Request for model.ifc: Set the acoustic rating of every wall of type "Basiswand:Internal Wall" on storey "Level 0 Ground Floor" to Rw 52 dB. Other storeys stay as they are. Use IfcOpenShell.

First a look at what the model holds.

```python
import ifcopenshell
import ifcopenshell.util.element

model = ifcopenshell.open("model.ifc")
print(model.schema)
storey = next(s for s in model.by_type("IfcBuildingStorey") if s.Name == "Level 0 Ground Floor")
walls = [e for e in ifcopenshell.util.element.get_decomposition(storey) if e.is_a("IfcWall")]
seen = {}
for e in walls:
    element_type = ifcopenshell.util.element.get_type(e)
    key = (element_type.Name if element_type != e and element_type else None, ifcopenshell.util.element.get_pset(e, "Pset_WallCommon", "AcousticRating"))
    seen[key] = seen.get(key, 0) + 1
for (name, value), count in sorted(seen.items(), key=str):
    print(count, "x", name, "|", value)
```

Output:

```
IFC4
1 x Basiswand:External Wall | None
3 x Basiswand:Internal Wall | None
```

```python
import ifcopenshell
import ifcopenshell.api.pset
import ifcopenshell.util.element

model = ifcopenshell.open("model.ifc")

storey = next(s for s in model.by_type("IfcBuildingStorey") if s.Name == "Level 0 Ground Floor")
walls = [e for e in ifcopenshell.util.element.get_decomposition(storey) if e.is_a("IfcWall")]

count = 0
for e in walls:
    element_type = ifcopenshell.util.element.get_type(e)
    if element_type in (None, e) or element_type.Name != "Basiswand:Internal Wall":
        continue
    # add_pset returns the element's existing set when there is one.
    pset = ifcopenshell.api.pset.add_pset(model, product=e, name="Pset_WallCommon")
    ifcopenshell.api.pset.edit_pset(model, pset=pset, properties={"AcousticRating": "Rw 52 dB"})
    count += 1

print(count, "walls updated")

model.write("model_rev.ifc")
```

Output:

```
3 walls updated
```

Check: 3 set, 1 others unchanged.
